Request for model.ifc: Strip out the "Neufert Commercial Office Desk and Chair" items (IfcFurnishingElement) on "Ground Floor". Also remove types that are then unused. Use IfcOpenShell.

First a look at what the model holds.

```python
import ifcopenshell
import ifcopenshell.util.element

model = ifcopenshell.open("model.ifc")
print(model.schema)
storey = next(s for s in model.by_type("IfcBuildingStorey") if s.Name == "Ground Floor")
furniture = [e for e in ifcopenshell.util.element.get_decomposition(storey) if e.is_a("IfcFurnishingElement")]
seen = {}
for e in furniture:
    element_type = ifcopenshell.util.element.get_type(e)
    name = element_type.Name if element_type not in (None, e) else None
    seen[name] = seen.get(name, 0) + 1
for name, count in sorted(seen.items(), key=str):
    print(count, "x", name)
```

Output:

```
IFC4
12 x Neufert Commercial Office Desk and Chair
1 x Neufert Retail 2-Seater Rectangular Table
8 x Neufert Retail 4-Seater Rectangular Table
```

```python
import ifcopenshell
import ifcopenshell.api.root
import ifcopenshell.util.element

model = ifcopenshell.open("model.ifc")

storey = next(s for s in model.by_type("IfcBuildingStorey") if s.Name == "Ground Floor")
furniture = [e for e in ifcopenshell.util.element.get_decomposition(storey) if e.is_a("IfcFurnishingElement")]
targets = [e for e in furniture if (t := ifcopenshell.util.element.get_type(e)) not in (None, e) and t.Name == "Neufert Commercial Office Desk and Chair"]
types = {ifcopenshell.util.element.get_type(e) for e in targets} - {None, *targets}

for e in targets:
    ifcopenshell.api.root.remove_product(model, product=e)
print(len(targets), "removed")

unused = [t for t in types if not ifcopenshell.util.element.get_types(t)]
for t in unused:
    ifcopenshell.api.root.remove_product(model, product=t)
print(len(unused), "unused types removed")

model.write("model_rev.ifc")
```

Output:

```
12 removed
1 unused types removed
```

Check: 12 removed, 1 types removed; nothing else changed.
